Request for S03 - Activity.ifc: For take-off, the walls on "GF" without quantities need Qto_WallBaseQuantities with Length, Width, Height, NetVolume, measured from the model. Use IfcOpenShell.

First a look at what the model holds.

```python
import ifcopenshell
import ifcopenshell.util.element
import ifcopenshell.util.unit

model = ifcopenshell.open("S03 - Activity.ifc")
print(model.schema)
for unit_type in ("LENGTHUNIT", "AREAUNIT", "VOLUMEUNIT"):
    print(unit_type, ifcopenshell.util.unit.calculate_unit_scale(model, unit_type))
storey = next(s for s in model.by_type("IfcBuildingStorey") if s.Name == "GF")
walls = [e for e in ifcopenshell.util.element.get_decomposition(storey) if e.is_a("IfcWall")]
for e in sorted(walls, key=lambda e: e.id()):
    print(e.id(), e.is_a(), e.Name, list(ifcopenshell.util.element.get_psets(e, qtos_only=True)), sep=" | ")
```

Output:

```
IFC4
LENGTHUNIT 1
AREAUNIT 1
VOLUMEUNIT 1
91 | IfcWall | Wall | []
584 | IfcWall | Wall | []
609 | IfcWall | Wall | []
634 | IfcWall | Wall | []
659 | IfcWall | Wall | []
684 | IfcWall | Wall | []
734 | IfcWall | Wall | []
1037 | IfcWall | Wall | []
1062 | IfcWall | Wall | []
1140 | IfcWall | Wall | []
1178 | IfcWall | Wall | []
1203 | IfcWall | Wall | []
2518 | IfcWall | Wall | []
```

```python
import ifcopenshell
import ifcopenshell.api.pset
import ifcopenshell.geom
import ifcopenshell.util.element
import ifcopenshell.util.shape
import ifcopenshell.util.unit

model = ifcopenshell.open("S03 - Activity.ifc")
unit_scale = ifcopenshell.util.unit.calculate_unit_scale(model)
volume_scale = ifcopenshell.util.unit.calculate_unit_scale(model, "VOLUMEUNIT")
settings = ifcopenshell.geom.settings()

storey = next(s for s in model.by_type("IfcBuildingStorey") if s.Name == "GF")
walls = [e for e in ifcopenshell.util.element.get_decomposition(storey) if e.is_a("IfcWall")]

for e in sorted(walls, key=lambda e: e.id()):
    if ifcopenshell.util.element.get_psets(e, qtos_only=True, should_inherit=False):
        continue
    # Geometry comes back in metres, in the element's own axes.
    shape = ifcopenshell.geom.create_shape(settings, e)
    values = {
        "Length": ifcopenshell.util.shape.get_x(shape.geometry) / unit_scale,
        "Width": ifcopenshell.util.shape.get_y(shape.geometry) / unit_scale,
        "Height": ifcopenshell.util.shape.get_z(shape.geometry) / unit_scale,
        "NetVolume": ifcopenshell.util.shape.get_volume(shape.geometry) / volume_scale,
    }
    qto = ifcopenshell.api.pset.add_qto(model, product=e, name="Qto_WallBaseQuantities")
    ifcopenshell.api.pset.edit_qto(model, qto=qto, properties=values)
    print(e.id(), {k: round(v, 3) for k, v in values.items()})

model.write("S03 - Activity_edited.ifc")
```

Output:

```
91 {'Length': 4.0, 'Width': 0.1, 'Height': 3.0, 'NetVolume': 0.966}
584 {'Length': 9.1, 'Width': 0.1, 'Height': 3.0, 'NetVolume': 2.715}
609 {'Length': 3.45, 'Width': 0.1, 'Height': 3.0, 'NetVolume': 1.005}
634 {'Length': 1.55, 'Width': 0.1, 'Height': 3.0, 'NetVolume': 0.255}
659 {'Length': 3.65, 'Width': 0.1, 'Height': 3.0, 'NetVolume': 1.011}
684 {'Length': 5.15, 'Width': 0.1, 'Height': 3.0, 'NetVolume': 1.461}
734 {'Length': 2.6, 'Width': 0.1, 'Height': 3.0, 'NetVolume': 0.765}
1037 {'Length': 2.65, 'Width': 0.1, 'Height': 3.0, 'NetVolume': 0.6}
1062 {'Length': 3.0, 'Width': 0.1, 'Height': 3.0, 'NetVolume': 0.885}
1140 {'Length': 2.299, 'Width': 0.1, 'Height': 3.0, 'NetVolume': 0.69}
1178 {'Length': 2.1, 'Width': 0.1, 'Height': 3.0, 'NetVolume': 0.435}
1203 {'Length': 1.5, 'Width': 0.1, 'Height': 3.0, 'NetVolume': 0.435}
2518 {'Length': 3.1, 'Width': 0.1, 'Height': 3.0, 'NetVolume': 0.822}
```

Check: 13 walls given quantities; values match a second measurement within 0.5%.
